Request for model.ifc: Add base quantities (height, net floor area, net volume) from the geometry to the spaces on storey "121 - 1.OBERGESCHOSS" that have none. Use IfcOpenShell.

First a look at what the model holds.

```python
import ifcopenshell
import ifcopenshell.util.element
import ifcopenshell.util.unit

model = ifcopenshell.open("model.ifc")
print(model.schema)
for unit_type in ("LENGTHUNIT", "AREAUNIT", "VOLUMEUNIT"):
    print(unit_type, ifcopenshell.util.unit.calculate_unit_scale(model, unit_type))
storey = next(s for s in model.by_type("IfcBuildingStorey") if s.Name == "121 - 1.OBERGESCHOSS")
spaces = [e for e in ifcopenshell.util.element.get_decomposition(storey) if e.is_a("IfcSpace")]
for e in sorted(spaces, key=lambda e: e.id()):
    print(e.id(), e.is_a(), e.Name, list(ifcopenshell.util.element.get_psets(e, qtos_only=True)), sep=" | ")
```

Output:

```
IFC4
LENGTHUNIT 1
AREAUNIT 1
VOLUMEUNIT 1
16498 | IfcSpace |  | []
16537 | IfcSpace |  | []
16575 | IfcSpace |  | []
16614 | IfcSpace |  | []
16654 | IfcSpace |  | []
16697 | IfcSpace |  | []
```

```python
import ifcopenshell
import ifcopenshell.api.pset
import ifcopenshell.geom
import ifcopenshell.util.element
import ifcopenshell.util.shape
import ifcopenshell.util.unit

model = ifcopenshell.open("model.ifc")
unit_scale = ifcopenshell.util.unit.calculate_unit_scale(model)
area_scale = ifcopenshell.util.unit.calculate_unit_scale(model, "AREAUNIT")
volume_scale = ifcopenshell.util.unit.calculate_unit_scale(model, "VOLUMEUNIT")
settings = ifcopenshell.geom.settings()

storey = next(s for s in model.by_type("IfcBuildingStorey") if s.Name == "121 - 1.OBERGESCHOSS")
spaces = [e for e in ifcopenshell.util.element.get_decomposition(storey) if e.is_a("IfcSpace")]

for e in sorted(spaces, key=lambda e: e.id()):
    if ifcopenshell.util.element.get_psets(e, qtos_only=True, should_inherit=False):
        continue
    # Geometry comes back in metres, in the element's own axes.
    shape = ifcopenshell.geom.create_shape(settings, e)
    values = {
        "Height": ifcopenshell.util.shape.get_z(shape.geometry) / unit_scale,
        "NetFloorArea": ifcopenshell.util.shape.get_footprint_area(shape.geometry) / area_scale,
        "NetVolume": ifcopenshell.util.shape.get_volume(shape.geometry) / volume_scale,
    }
    qto = ifcopenshell.api.pset.add_qto(model, product=e, name="Qto_SpaceBaseQuantities")
    ifcopenshell.api.pset.edit_qto(model, qto=qto, properties=values)
    print(e.id(), {k: round(v, 3) for k, v in values.items()})

model.write("model-out.ifc")
```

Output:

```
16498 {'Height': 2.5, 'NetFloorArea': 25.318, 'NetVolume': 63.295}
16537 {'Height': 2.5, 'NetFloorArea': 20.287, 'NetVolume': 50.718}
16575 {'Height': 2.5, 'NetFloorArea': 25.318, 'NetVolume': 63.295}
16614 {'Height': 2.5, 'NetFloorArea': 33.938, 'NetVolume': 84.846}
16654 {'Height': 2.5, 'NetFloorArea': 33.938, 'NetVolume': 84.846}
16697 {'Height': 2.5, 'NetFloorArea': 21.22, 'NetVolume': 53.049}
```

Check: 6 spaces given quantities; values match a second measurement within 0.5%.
